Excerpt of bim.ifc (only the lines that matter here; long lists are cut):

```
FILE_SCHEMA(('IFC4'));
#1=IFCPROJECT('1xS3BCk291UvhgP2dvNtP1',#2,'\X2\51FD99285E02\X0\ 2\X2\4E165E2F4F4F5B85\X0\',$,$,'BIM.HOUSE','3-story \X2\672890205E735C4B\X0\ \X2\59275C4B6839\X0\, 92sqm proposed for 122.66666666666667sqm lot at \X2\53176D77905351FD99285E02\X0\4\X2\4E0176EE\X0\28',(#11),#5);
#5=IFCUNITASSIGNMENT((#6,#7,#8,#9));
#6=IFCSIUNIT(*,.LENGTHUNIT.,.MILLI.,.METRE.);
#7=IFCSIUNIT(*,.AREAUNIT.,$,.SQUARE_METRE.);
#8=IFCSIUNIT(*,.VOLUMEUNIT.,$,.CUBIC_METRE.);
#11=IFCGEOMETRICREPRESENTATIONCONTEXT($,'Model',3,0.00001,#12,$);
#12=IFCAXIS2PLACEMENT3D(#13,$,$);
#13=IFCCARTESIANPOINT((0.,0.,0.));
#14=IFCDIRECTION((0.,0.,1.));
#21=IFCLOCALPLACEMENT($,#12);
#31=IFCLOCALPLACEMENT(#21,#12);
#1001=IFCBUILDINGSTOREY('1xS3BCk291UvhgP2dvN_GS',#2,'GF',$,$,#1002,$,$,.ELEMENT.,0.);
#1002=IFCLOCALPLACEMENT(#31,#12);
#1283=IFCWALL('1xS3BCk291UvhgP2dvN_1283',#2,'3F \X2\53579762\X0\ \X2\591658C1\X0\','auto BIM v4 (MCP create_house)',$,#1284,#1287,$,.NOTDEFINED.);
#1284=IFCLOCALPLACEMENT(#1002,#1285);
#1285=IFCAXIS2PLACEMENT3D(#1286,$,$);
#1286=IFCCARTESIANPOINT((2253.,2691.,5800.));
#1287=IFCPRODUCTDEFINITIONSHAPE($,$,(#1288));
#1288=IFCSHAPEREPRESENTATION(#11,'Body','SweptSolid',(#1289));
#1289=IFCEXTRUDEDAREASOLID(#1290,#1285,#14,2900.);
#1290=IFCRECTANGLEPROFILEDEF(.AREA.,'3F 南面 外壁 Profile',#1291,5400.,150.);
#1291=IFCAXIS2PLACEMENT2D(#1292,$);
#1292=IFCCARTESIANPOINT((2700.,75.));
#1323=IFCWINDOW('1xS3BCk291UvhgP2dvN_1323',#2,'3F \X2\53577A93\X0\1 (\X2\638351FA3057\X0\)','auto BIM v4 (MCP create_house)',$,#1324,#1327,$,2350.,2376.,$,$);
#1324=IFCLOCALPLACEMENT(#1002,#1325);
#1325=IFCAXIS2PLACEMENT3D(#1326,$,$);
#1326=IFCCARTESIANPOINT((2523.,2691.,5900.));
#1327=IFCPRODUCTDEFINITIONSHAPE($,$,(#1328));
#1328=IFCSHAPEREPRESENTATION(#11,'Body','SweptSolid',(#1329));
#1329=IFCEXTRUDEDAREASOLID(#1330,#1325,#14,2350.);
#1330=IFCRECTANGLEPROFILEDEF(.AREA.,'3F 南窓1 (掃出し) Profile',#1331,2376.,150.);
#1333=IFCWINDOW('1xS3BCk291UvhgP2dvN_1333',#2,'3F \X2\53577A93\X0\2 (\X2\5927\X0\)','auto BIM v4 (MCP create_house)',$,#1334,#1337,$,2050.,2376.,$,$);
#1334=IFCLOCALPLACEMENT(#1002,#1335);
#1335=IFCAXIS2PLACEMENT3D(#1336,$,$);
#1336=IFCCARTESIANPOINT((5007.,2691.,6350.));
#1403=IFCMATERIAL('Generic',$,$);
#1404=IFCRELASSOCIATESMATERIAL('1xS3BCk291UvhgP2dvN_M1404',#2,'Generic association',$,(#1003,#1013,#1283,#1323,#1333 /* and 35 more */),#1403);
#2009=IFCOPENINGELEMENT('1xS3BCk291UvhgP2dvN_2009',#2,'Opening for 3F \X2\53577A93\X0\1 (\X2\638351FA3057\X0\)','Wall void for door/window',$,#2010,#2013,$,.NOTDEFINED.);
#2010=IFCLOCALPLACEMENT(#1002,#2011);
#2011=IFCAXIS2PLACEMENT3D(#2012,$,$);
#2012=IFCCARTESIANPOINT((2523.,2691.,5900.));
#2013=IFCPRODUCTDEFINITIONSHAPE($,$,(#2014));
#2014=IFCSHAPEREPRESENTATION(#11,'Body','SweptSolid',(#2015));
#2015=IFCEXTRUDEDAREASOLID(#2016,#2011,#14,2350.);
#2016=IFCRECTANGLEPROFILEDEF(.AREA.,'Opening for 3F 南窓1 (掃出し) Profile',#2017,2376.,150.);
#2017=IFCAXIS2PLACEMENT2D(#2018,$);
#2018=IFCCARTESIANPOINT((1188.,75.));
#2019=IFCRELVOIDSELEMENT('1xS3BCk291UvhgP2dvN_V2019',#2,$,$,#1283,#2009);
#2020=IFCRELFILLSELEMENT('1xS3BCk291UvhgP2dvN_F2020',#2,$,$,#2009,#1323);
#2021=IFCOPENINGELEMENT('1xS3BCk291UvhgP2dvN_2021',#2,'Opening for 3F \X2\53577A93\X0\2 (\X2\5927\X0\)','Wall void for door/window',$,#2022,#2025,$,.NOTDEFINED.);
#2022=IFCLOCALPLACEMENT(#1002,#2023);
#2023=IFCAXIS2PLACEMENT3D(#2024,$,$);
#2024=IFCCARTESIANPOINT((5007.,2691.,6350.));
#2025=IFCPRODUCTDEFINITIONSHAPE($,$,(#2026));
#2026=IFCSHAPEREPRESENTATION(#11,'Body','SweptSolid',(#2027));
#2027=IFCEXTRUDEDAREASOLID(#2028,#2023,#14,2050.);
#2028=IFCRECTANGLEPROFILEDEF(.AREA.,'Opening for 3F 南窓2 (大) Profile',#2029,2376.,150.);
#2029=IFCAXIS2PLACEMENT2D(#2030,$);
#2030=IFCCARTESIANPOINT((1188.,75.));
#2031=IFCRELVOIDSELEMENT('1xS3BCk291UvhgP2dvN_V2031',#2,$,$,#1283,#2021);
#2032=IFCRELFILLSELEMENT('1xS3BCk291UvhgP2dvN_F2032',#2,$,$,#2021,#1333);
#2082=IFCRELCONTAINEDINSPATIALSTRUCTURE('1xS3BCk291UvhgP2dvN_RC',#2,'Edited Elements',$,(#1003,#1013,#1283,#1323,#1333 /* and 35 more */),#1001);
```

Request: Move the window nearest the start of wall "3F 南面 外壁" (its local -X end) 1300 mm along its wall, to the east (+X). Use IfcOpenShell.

```python
import ifcopenshell
import ifcopenshell.api.geometry
import ifcopenshell.util.placement

model = ifcopenshell.open("bim.ifc")

window = model.by_guid("1xS3BCk291UvhgP2dvN_1323")
opening = window.FillsVoids[0].RelatingOpeningElement
wall = opening.VoidsElements[0].RelatingBuildingElement

wall_matrix = ifcopenshell.util.placement.get_local_placement(wall.ObjectPlacement)
shift = wall_matrix[:3, 0] * 1300.0
before = ifcopenshell.util.placement.get_local_placement(window.ObjectPlacement)[:3, 3].copy()

# The window is not placed relative to its opening, so move both.
for product in (opening, window):
    matrix = ifcopenshell.util.placement.get_local_placement(product.ObjectPlacement)
    matrix[:3, 3] += shift
    ifcopenshell.api.geometry.edit_object_placement(model, product=product, matrix=matrix, is_si=False)

after = ifcopenshell.util.placement.get_local_placement(window.ObjectPlacement)[:3, 3]
print("window moved by", (after - before).round(3) + 0.0)

model.write("bim_rev.ifc")
```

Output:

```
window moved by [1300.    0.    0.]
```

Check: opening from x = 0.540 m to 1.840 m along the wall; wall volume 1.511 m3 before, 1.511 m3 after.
